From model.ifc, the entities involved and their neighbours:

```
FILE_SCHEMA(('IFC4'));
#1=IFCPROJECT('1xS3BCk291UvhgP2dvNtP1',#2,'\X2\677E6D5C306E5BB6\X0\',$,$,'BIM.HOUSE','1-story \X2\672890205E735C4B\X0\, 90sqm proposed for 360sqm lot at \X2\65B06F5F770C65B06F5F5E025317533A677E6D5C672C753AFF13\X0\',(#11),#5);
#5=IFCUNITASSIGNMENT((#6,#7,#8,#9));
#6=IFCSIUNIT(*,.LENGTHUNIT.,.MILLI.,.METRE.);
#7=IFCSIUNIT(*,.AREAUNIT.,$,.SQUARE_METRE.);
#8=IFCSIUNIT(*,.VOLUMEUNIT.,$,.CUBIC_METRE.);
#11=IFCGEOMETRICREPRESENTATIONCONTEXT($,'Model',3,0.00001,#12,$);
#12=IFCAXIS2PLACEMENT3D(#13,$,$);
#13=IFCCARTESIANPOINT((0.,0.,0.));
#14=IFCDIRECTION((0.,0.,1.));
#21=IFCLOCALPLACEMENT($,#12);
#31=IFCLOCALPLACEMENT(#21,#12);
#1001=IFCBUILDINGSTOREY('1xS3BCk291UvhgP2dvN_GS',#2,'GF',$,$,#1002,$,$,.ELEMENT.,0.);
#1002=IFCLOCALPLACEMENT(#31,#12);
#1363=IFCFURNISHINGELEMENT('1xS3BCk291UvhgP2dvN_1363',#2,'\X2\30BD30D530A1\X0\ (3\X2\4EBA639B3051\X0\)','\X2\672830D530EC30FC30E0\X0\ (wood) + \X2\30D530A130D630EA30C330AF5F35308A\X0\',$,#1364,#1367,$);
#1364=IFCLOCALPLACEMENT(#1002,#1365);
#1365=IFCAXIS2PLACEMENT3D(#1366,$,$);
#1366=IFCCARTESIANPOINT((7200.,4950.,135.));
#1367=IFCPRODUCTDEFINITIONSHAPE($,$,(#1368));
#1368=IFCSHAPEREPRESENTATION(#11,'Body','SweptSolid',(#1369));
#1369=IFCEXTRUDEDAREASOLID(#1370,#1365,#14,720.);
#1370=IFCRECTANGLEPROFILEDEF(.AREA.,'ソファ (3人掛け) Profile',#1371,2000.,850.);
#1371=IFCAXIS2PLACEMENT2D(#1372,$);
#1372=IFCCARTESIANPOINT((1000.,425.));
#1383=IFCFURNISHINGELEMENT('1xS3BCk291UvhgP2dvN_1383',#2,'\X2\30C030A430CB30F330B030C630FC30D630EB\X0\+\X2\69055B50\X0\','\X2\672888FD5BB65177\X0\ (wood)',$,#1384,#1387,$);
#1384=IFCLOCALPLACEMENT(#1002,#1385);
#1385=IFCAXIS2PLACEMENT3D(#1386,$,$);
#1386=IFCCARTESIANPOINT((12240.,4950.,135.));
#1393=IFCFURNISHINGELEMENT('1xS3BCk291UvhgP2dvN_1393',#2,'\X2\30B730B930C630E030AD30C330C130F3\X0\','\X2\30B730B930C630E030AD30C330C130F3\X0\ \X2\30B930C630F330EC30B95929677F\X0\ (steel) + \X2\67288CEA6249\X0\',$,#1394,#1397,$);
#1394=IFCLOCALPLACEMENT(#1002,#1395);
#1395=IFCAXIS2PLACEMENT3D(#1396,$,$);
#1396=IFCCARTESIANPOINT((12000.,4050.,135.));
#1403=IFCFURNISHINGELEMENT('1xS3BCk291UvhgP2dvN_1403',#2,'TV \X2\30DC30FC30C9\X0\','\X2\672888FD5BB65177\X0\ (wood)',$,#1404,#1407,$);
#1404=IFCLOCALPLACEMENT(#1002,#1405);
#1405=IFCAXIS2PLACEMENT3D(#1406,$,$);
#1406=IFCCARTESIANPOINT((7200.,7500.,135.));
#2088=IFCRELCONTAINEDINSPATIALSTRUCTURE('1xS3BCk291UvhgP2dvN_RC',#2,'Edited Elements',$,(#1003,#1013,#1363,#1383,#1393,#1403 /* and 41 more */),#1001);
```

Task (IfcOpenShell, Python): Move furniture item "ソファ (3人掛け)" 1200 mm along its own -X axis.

```python
import ifcopenshell
import ifcopenshell.api.geometry
import ifcopenshell.util.placement
import ifcopenshell.util.unit

model = ifcopenshell.open("model.ifc")
unit_scale = ifcopenshell.util.unit.calculate_unit_scale(model)

item = model.by_guid("1xS3BCk291UvhgP2dvN_1363")
matrix = ifcopenshell.util.placement.get_local_placement(item.ObjectPlacement)
matrix[:3, 3] -= matrix[:3, 0] * 1.2 / unit_scale
ifcopenshell.api.geometry.edit_object_placement(model, product=item, matrix=matrix, is_si=False)

print(ifcopenshell.util.placement.get_local_placement(item.ObjectPlacement).round(3) + 0.0)

model.write("model_rev.ifc")
```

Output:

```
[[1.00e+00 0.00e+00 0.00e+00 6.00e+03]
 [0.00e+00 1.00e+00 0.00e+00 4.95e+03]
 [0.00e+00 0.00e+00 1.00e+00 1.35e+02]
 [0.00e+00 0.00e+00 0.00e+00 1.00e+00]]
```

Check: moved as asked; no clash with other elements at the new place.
